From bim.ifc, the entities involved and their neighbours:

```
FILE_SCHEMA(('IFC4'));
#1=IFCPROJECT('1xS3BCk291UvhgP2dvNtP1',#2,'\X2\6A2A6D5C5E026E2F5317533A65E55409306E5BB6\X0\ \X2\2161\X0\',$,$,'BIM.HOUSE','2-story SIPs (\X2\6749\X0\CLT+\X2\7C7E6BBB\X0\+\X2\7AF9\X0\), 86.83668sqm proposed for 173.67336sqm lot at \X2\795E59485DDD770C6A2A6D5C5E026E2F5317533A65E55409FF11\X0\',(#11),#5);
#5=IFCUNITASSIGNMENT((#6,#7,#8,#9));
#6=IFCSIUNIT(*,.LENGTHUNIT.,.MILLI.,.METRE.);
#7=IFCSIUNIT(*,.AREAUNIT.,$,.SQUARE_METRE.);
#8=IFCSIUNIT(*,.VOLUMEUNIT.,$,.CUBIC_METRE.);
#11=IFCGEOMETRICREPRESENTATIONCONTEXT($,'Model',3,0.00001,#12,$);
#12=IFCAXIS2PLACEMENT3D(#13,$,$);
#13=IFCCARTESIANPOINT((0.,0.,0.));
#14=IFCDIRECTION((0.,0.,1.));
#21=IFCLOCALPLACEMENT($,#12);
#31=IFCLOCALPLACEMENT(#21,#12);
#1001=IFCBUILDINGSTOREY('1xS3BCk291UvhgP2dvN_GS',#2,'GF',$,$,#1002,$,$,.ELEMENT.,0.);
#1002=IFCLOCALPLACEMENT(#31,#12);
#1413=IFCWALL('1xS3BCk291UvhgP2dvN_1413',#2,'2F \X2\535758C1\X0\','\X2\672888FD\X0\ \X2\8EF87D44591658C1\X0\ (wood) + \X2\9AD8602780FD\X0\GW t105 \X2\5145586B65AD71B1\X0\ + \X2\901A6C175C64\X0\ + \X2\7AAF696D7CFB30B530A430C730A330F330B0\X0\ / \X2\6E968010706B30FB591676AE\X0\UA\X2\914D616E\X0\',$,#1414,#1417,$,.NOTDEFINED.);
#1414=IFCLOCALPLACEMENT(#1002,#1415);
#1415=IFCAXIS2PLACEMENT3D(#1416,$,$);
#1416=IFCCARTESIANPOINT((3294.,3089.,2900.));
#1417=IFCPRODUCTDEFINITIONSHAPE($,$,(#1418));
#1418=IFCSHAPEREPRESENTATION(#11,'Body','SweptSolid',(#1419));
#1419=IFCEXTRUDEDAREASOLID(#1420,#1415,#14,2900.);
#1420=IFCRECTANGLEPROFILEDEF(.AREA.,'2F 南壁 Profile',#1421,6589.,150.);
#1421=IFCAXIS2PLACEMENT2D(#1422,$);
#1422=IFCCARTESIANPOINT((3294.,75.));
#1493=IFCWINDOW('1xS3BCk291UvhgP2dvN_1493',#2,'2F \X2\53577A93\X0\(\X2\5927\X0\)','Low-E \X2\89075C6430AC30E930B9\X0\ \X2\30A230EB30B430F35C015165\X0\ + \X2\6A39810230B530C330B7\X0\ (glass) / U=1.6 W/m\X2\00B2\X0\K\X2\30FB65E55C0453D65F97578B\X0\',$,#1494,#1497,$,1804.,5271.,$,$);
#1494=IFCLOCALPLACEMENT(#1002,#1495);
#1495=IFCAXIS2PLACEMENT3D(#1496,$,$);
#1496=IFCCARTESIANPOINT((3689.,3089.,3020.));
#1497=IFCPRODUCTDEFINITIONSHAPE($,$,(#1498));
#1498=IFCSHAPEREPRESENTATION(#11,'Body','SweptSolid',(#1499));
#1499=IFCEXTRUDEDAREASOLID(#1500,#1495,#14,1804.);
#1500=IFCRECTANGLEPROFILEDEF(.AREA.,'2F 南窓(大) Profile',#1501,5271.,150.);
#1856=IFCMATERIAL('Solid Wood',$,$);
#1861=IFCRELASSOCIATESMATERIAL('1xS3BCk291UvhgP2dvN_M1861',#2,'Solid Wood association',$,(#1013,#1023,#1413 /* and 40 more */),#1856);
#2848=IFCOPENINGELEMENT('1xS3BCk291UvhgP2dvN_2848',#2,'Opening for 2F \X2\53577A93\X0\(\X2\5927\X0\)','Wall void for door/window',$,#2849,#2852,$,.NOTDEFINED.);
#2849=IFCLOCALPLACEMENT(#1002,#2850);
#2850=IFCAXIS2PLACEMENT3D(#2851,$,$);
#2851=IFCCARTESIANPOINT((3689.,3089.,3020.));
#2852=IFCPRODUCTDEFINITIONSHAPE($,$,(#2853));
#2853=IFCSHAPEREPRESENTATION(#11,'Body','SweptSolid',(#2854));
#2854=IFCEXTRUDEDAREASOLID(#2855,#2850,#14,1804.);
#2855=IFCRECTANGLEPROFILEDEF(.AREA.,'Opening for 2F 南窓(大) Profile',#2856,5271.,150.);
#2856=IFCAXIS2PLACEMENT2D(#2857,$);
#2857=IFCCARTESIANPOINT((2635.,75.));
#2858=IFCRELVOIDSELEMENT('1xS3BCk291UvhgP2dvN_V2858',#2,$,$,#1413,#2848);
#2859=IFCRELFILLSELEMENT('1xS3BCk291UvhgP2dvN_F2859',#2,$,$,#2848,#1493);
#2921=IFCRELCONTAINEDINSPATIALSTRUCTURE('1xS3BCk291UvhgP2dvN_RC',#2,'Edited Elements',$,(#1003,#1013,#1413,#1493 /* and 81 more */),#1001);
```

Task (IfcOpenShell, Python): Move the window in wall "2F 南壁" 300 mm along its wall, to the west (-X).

```python
import ifcopenshell
import ifcopenshell.api.geometry
import ifcopenshell.util.placement

model = ifcopenshell.open("bim.ifc")

window = model.by_guid("1xS3BCk291UvhgP2dvN_1493")
opening = window.FillsVoids[0].RelatingOpeningElement
wall = opening.VoidsElements[0].RelatingBuildingElement

wall_matrix = ifcopenshell.util.placement.get_local_placement(wall.ObjectPlacement)
shift = wall_matrix[:3, 0] * -300.0
before = ifcopenshell.util.placement.get_local_placement(window.ObjectPlacement)[:3, 3].copy()

# The window is not placed relative to its opening, so move both.
for product in (opening, window):
    matrix = ifcopenshell.util.placement.get_local_placement(product.ObjectPlacement)
    matrix[:3, 3] += shift
    ifcopenshell.api.geometry.edit_object_placement(model, product=product, matrix=matrix, is_si=False)

after = ifcopenshell.util.placement.get_local_placement(window.ObjectPlacement)[:3, 3]
print("window moved by", (after - before).round(3) + 0.0)

model.write("bim_v2.ifc")
```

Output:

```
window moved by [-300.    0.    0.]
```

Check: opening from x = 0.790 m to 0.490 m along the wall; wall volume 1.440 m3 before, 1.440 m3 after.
